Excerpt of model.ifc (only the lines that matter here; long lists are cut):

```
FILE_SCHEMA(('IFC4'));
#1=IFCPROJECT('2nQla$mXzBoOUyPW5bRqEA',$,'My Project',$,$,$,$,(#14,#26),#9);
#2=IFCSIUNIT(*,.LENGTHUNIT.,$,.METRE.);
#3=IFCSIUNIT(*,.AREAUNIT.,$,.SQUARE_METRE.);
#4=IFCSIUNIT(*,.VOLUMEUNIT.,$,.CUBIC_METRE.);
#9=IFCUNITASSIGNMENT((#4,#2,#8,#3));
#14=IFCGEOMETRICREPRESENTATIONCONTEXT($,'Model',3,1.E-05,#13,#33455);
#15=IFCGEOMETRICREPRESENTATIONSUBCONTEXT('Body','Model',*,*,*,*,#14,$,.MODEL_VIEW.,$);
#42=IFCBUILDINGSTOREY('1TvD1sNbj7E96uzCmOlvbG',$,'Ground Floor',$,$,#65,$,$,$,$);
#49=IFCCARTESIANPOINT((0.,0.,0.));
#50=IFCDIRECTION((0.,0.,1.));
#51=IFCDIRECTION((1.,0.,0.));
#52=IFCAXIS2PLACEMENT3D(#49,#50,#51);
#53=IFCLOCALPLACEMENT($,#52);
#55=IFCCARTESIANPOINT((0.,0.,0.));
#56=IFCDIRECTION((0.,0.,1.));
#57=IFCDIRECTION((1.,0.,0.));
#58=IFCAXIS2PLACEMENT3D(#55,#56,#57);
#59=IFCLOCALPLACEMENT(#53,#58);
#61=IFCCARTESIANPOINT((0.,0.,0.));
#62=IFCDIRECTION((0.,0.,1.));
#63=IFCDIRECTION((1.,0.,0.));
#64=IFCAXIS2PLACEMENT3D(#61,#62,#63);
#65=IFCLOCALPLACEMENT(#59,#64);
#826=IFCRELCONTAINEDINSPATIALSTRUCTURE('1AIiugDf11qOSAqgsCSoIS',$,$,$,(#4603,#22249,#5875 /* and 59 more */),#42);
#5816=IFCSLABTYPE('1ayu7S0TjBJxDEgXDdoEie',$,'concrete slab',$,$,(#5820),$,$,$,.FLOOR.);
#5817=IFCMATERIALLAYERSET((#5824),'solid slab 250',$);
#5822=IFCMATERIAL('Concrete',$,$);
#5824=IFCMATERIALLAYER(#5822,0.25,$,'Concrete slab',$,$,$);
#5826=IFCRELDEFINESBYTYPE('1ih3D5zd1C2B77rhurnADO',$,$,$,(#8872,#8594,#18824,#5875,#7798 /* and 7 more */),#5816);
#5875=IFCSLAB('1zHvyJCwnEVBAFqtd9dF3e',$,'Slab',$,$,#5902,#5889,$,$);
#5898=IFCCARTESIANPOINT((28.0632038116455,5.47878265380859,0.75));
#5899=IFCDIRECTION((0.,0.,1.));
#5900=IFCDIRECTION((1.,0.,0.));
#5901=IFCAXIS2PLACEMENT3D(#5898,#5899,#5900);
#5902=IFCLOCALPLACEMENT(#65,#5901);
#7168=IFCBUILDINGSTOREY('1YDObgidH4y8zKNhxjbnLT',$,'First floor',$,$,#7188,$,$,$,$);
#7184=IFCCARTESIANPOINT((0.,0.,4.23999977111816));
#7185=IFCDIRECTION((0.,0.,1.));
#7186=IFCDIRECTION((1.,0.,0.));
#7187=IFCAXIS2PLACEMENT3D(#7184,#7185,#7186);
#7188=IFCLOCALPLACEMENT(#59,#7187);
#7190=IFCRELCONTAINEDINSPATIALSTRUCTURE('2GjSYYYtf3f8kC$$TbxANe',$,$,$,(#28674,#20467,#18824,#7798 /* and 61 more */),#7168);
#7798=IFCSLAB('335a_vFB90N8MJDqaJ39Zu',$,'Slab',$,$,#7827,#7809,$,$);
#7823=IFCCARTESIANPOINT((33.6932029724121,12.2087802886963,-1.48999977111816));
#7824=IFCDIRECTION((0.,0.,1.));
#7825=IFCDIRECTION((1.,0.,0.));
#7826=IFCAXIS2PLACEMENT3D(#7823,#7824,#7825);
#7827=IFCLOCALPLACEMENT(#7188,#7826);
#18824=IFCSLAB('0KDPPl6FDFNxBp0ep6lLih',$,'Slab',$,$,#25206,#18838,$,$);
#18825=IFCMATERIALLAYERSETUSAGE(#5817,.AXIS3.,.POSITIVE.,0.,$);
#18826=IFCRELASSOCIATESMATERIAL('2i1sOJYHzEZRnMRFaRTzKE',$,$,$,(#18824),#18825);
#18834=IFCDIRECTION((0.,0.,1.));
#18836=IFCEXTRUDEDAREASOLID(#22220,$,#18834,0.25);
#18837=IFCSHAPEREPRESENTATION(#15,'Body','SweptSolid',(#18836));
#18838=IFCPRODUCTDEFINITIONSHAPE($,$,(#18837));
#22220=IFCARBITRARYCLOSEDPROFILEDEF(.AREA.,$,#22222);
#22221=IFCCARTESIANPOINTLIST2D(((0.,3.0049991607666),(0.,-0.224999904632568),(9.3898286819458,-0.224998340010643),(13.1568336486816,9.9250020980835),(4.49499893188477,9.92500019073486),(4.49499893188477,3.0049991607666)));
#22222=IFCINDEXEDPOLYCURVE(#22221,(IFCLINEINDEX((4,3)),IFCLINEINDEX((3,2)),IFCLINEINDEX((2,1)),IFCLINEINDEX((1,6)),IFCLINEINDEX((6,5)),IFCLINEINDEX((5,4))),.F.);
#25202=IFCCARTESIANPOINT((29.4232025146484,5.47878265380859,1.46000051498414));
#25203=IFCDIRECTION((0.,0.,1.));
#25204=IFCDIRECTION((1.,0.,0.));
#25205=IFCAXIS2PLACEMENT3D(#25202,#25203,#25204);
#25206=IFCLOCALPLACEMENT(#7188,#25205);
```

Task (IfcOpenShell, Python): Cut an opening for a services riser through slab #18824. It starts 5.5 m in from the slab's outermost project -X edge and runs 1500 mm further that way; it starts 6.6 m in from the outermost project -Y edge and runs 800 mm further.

```python
import numpy as np
import ifcopenshell
import ifcopenshell.api.feature
import ifcopenshell.api.geometry
import ifcopenshell.api.root
import ifcopenshell.geom
import ifcopenshell.util.placement
import ifcopenshell.util.representation
import ifcopenshell.util.shape
import ifcopenshell.util.unit

model = ifcopenshell.open("model.ifc")
unit_scale = ifcopenshell.util.unit.calculate_unit_scale(model)
settings = ifcopenshell.geom.settings()


def volume(element):
    """Net volume in cubic metres, openings subtracted."""
    shape = ifcopenshell.geom.create_shape(settings, element)
    return ifcopenshell.util.shape.get_volume(shape.geometry)


slab = model.by_guid("0KDPPl6FDFNxBp0ep6lLih")
before = volume(slab)

# Extent in the slab's own axes, in metres. The edges named are its -X and -Y sides.
slab_shape = ifcopenshell.geom.create_shape(settings, slab)
vertices = ifcopenshell.util.shape.get_vertices(slab_shape.geometry)
x_min, y_min, bottom = vertices.min(axis=0)
top = vertices[:, 2].max()

opening = ifcopenshell.api.root.create_entity(model, ifc_class="IfcOpeningElement", name="Services riser opening", predefined_type="OPENING")
context = ifcopenshell.util.representation.get_context(model, "Model", "Body", "MODEL_VIEW")
width, depth = 1.5, 0.8
outline = [(0.0, 0.0), (width, 0.0), (width, depth), (0.0, depth), (0.0, 0.0)]
# Overshoot both faces by 50 mm so the cut is clean.
shape = ifcopenshell.api.geometry.add_slab_representation(
    model, context=context, depth=top - bottom + 0.1, polyline=outline
)
ifcopenshell.api.geometry.assign_representation(model, product=opening, representation=shape)

matrix = ifcopenshell.util.placement.get_local_placement(slab.ObjectPlacement)
matrix[:, 3] = matrix @ np.append(np.array([x_min + 5.5, y_min + 6.6, bottom - 0.05]) / unit_scale, 1.0)
ifcopenshell.api.geometry.edit_object_placement(model, product=opening, matrix=matrix, is_si=False)
ifcopenshell.api.feature.add_feature(model, feature=opening, element=slab)

after = volume(slab)

print(f"slab volume {before:.3f} -> {after:.3f} m3")

model.write("model_v2.ifc")
```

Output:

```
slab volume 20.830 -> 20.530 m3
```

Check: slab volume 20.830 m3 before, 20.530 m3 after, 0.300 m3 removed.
